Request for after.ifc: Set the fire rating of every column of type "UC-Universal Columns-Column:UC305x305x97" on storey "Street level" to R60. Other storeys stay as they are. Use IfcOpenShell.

First a look at what the model holds.

```python
import ifcopenshell
import ifcopenshell.util.element

model = ifcopenshell.open("after.ifc")
print(model.schema)
storey = next(s for s in model.by_type("IfcBuildingStorey") if s.Name == "Street level")
columns = [e for e in ifcopenshell.util.element.get_decomposition(storey) if e.is_a("IfcColumn")]
seen = {}
for e in columns:
    element_type = ifcopenshell.util.element.get_type(e)
    key = (element_type.Name if element_type != e and element_type else None, ifcopenshell.util.element.get_pset(e, "Pset_ColumnCommon", "FireRating"))
    seen[key] = seen.get(key, 0) + 1
for (name, value), count in sorted(seen.items(), key=str):
    print(count, "x", name, "|", value)
```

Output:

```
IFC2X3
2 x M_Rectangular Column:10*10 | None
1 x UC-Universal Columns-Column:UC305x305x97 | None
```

```python
import ifcopenshell
import ifcopenshell.api.pset
import ifcopenshell.util.element

model = ifcopenshell.open("after.ifc")

storey = next(s for s in model.by_type("IfcBuildingStorey") if s.Name == "Street level")
columns = [e for e in ifcopenshell.util.element.get_decomposition(storey) if e.is_a("IfcColumn")]

count = 0
for e in columns:
    element_type = ifcopenshell.util.element.get_type(e)
    if element_type in (None, e) or element_type.Name != "UC-Universal Columns-Column:UC305x305x97":
        continue
    # add_pset returns the element's existing set when there is one.
    pset = ifcopenshell.api.pset.add_pset(model, product=e, name="Pset_ColumnCommon")
    ifcopenshell.api.pset.edit_pset(model, pset=pset, properties={"FireRating": "R60"})
    count += 1

print(count, "columns updated")

model.write("after_rev.ifc")
```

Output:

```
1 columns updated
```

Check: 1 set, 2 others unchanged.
